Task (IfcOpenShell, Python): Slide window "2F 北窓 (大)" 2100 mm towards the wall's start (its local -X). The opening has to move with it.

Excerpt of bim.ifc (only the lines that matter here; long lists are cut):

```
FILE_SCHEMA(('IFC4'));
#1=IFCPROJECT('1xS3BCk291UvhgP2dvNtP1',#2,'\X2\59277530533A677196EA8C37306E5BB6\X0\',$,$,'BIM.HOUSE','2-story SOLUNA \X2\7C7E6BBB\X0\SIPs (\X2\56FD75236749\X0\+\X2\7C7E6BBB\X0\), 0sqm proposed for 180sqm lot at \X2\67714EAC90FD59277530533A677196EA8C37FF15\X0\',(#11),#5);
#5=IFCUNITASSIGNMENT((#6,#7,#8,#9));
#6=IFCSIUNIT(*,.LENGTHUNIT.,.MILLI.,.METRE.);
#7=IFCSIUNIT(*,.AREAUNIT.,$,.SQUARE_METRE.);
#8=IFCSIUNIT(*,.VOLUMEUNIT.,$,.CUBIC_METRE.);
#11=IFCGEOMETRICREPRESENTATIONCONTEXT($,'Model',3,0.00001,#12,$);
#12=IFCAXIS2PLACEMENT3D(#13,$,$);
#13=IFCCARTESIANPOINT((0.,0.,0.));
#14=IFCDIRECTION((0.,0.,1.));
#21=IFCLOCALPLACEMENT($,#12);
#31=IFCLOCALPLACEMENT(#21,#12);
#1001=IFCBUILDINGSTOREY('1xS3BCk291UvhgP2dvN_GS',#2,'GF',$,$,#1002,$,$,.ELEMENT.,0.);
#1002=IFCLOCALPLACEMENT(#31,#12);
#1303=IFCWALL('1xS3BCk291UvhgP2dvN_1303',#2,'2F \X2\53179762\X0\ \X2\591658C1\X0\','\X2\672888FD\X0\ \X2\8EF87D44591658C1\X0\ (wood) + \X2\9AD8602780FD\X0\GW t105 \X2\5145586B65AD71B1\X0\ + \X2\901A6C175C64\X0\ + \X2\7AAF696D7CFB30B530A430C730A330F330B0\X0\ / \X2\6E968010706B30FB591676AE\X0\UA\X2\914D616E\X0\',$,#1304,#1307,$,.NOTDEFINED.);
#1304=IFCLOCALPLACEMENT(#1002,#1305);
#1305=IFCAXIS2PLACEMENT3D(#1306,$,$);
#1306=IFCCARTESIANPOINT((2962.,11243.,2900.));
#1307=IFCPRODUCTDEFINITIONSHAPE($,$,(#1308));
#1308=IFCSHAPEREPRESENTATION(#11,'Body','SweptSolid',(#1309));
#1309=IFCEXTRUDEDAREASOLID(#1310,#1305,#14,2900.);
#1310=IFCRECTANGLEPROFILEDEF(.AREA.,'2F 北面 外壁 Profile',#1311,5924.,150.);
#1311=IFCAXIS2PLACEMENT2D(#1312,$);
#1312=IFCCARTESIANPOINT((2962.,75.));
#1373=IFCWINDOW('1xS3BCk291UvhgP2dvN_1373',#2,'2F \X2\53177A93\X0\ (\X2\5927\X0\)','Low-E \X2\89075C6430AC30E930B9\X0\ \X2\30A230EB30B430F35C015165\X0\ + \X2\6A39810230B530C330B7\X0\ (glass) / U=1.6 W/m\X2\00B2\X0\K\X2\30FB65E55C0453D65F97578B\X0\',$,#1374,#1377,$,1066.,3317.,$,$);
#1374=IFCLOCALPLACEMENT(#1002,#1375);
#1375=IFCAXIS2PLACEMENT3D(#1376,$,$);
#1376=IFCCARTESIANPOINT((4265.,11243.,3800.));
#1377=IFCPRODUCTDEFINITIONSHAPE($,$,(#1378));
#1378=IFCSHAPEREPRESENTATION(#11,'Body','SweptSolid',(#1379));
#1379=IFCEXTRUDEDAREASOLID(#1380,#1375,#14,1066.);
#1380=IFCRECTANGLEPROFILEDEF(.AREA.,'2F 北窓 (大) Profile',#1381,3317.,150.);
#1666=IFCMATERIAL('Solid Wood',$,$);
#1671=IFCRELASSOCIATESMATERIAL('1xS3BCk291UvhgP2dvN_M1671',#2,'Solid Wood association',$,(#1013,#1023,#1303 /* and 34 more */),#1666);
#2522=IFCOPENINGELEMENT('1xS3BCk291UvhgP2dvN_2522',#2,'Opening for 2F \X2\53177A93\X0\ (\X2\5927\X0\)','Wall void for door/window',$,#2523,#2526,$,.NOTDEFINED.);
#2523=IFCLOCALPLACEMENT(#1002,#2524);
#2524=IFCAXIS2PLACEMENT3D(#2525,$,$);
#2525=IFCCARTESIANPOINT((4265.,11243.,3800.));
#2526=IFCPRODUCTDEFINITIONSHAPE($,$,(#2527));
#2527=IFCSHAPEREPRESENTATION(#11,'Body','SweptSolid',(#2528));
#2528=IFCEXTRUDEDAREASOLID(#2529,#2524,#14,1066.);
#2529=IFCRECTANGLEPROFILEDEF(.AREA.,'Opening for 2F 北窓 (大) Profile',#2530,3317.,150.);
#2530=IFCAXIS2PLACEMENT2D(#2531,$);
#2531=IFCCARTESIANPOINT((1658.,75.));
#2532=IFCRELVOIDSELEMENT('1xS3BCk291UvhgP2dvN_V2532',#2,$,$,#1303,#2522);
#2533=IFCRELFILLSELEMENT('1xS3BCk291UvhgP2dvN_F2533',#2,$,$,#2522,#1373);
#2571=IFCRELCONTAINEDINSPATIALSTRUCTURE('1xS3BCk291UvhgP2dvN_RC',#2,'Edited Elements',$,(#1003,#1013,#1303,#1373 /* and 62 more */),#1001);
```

```python
import ifcopenshell
import ifcopenshell.api.geometry
import ifcopenshell.util.placement
import ifcopenshell.util.unit

model = ifcopenshell.open("bim.ifc")
unit_scale = ifcopenshell.util.unit.calculate_unit_scale(model)

window = model.by_guid("1xS3BCk291UvhgP2dvN_1373")
opening = window.FillsVoids[0].RelatingOpeningElement
wall = opening.VoidsElements[0].RelatingBuildingElement

wall_matrix = ifcopenshell.util.placement.get_local_placement(wall.ObjectPlacement)
shift = wall_matrix[:3, 0] * -2.1 / unit_scale
before = ifcopenshell.util.placement.get_local_placement(window.ObjectPlacement)[:3, 3].copy()

# The window is not placed relative to its opening, so move both.
for product in (opening, window):
    matrix = ifcopenshell.util.placement.get_local_placement(product.ObjectPlacement)
    matrix[:3, 3] += shift
    ifcopenshell.api.geometry.edit_object_placement(model, product=product, matrix=matrix, is_si=False)

after = ifcopenshell.util.placement.get_local_placement(window.ObjectPlacement)[:3, 3]
print("window moved by", (after - before).round(3) + 0.0)

model.write("bim_updated.ifc")
```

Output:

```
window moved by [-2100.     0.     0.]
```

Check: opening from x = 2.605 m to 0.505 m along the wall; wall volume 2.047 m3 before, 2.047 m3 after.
